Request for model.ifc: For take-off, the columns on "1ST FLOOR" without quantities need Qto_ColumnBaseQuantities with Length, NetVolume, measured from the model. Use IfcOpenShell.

First a look at what the model holds.

```python
import ifcopenshell
import ifcopenshell.util.element
import ifcopenshell.util.unit

model = ifcopenshell.open("model.ifc")
print(model.schema)
for unit_type in ("LENGTHUNIT", "AREAUNIT", "VOLUMEUNIT"):
    print(unit_type, ifcopenshell.util.unit.calculate_unit_scale(model, unit_type))
storey = next(s for s in model.by_type("IfcBuildingStorey") if s.Name == "1ST FLOOR")
columns = [e for e in ifcopenshell.util.element.get_decomposition(storey) if e.is_a("IfcColumn")]
for e in sorted(columns, key=lambda e: e.id()):
    print(e.id(), e.is_a(), e.Name, list(ifcopenshell.util.element.get_psets(e, qtos_only=True)), sep=" | ")
```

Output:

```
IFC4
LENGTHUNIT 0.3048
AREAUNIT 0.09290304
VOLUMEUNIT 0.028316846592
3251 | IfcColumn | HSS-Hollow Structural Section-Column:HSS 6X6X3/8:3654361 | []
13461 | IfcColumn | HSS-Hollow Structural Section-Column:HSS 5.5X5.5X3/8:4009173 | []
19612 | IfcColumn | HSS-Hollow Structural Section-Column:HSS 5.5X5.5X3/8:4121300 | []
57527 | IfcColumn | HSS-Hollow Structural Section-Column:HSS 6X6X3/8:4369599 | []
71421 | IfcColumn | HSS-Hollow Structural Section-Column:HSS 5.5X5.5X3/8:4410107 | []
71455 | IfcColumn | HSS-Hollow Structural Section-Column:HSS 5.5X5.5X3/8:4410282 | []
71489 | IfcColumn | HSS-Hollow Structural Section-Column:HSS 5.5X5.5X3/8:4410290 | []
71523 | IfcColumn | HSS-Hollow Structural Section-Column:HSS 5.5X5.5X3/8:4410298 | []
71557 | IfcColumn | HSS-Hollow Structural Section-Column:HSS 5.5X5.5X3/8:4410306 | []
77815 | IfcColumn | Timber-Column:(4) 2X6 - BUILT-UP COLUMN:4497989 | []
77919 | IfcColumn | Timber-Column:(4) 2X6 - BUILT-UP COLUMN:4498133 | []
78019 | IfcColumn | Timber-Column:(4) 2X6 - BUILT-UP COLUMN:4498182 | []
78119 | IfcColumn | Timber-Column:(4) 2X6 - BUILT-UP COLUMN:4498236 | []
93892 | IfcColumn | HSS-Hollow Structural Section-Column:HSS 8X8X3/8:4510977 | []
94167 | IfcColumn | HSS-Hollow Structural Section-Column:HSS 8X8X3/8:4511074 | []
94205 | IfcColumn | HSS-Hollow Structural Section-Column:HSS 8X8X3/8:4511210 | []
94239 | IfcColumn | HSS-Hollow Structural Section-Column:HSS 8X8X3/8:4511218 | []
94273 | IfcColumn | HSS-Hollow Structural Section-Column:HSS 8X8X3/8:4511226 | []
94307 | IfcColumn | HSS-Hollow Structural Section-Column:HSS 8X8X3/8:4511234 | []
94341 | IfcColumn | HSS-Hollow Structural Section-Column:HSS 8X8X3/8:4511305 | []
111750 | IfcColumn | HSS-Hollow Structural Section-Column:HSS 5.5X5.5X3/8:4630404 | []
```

```python
import ifcopenshell
import ifcopenshell.api.pset
import ifcopenshell.geom
import ifcopenshell.util.element
import ifcopenshell.util.shape
import ifcopenshell.util.unit

model = ifcopenshell.open("model.ifc")
unit_scale = ifcopenshell.util.unit.calculate_unit_scale(model)
volume_scale = ifcopenshell.util.unit.calculate_unit_scale(model, "VOLUMEUNIT")
settings = ifcopenshell.geom.settings()

storey = next(s for s in model.by_type("IfcBuildingStorey") if s.Name == "1ST FLOOR")
columns = [e for e in ifcopenshell.util.element.get_decomposition(storey) if e.is_a("IfcColumn")]

for e in sorted(columns, key=lambda e: e.id()):
    if ifcopenshell.util.element.get_psets(e, qtos_only=True, should_inherit=False):
        continue
    # Geometry comes back in metres, in the element's own axes.
    shape = ifcopenshell.geom.create_shape(settings, e)
    values = {
        "Length": ifcopenshell.util.shape.get_z(shape.geometry) / unit_scale,
        "NetVolume": ifcopenshell.util.shape.get_volume(shape.geometry) / volume_scale,
    }
    qto = ifcopenshell.api.pset.add_qto(model, product=e, name="Qto_ColumnBaseQuantities")
    ifcopenshell.api.pset.edit_qto(model, qto=qto, properties=values)
    print(e.id(), {k: round(v, 3) for k, v in values.items()})

model.write("model_v2.ifc")
```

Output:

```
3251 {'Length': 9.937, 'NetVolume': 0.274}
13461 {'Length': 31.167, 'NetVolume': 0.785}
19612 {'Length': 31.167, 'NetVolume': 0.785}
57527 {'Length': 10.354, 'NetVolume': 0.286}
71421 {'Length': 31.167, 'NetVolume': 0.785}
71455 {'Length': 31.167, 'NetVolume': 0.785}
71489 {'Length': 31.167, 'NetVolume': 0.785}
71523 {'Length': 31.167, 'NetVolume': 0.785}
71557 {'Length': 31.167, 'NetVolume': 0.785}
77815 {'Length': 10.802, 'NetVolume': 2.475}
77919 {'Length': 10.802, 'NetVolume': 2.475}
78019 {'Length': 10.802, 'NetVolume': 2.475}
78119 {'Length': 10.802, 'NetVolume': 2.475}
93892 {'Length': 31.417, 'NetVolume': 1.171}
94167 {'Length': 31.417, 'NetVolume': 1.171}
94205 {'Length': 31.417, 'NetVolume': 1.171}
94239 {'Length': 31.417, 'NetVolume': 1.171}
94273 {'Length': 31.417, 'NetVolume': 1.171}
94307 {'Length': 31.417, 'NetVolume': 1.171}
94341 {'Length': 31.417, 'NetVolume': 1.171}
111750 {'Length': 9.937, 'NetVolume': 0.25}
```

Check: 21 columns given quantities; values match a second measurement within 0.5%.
